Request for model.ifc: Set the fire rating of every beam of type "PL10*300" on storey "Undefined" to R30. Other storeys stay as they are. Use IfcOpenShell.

First a look at what the model holds.

```python
import ifcopenshell
import ifcopenshell.util.element

model = ifcopenshell.open("model.ifc")
print(model.schema)
storey = next(s for s in model.by_type("IfcBuildingStorey") if s.Name == "Undefined")
beams = [e for e in ifcopenshell.util.element.get_decomposition(storey) if e.is_a("IfcBeam")]
seen = {}
for e in beams:
    element_type = ifcopenshell.util.element.get_type(e)
    key = (element_type.Name if element_type != e and element_type else None, ifcopenshell.util.element.get_pset(e, "Pset_BeamCommon", "FireRating"))
    seen[key] = seen.get(key, 0) + 1
for (name, value), count in sorted(seen.items(), key=str):
    print(count, "x", name, "|", value)
```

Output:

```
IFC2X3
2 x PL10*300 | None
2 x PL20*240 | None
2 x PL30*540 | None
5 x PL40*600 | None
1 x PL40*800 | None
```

```python
import ifcopenshell
import ifcopenshell.api.pset
import ifcopenshell.util.element

model = ifcopenshell.open("model.ifc")

storey = next(s for s in model.by_type("IfcBuildingStorey") if s.Name == "Undefined")
beams = [e for e in ifcopenshell.util.element.get_decomposition(storey) if e.is_a("IfcBeam")]

count = 0
for e in beams:
    element_type = ifcopenshell.util.element.get_type(e)
    if element_type in (None, e) or element_type.Name != "PL10*300":
        continue
    found = ifcopenshell.util.element.get_pset(e, "Pset_BeamCommon", should_inherit=False)
    if found:
        pset = model.by_id(found["id"])
        if len(ifcopenshell.util.element.get_elements_by_pset(pset)) > 1:
            pset = ifcopenshell.api.pset.unshare_pset(model, products=[e], pset=pset)[0]
    else:
        pset = ifcopenshell.api.pset.add_pset(model, product=e, name="Pset_BeamCommon")
    ifcopenshell.api.pset.edit_pset(model, pset=pset, properties={"FireRating": "R30"})
    count += 1

print(count, "beams updated")

model.write("model_updated.ifc")
```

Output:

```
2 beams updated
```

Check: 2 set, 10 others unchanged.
